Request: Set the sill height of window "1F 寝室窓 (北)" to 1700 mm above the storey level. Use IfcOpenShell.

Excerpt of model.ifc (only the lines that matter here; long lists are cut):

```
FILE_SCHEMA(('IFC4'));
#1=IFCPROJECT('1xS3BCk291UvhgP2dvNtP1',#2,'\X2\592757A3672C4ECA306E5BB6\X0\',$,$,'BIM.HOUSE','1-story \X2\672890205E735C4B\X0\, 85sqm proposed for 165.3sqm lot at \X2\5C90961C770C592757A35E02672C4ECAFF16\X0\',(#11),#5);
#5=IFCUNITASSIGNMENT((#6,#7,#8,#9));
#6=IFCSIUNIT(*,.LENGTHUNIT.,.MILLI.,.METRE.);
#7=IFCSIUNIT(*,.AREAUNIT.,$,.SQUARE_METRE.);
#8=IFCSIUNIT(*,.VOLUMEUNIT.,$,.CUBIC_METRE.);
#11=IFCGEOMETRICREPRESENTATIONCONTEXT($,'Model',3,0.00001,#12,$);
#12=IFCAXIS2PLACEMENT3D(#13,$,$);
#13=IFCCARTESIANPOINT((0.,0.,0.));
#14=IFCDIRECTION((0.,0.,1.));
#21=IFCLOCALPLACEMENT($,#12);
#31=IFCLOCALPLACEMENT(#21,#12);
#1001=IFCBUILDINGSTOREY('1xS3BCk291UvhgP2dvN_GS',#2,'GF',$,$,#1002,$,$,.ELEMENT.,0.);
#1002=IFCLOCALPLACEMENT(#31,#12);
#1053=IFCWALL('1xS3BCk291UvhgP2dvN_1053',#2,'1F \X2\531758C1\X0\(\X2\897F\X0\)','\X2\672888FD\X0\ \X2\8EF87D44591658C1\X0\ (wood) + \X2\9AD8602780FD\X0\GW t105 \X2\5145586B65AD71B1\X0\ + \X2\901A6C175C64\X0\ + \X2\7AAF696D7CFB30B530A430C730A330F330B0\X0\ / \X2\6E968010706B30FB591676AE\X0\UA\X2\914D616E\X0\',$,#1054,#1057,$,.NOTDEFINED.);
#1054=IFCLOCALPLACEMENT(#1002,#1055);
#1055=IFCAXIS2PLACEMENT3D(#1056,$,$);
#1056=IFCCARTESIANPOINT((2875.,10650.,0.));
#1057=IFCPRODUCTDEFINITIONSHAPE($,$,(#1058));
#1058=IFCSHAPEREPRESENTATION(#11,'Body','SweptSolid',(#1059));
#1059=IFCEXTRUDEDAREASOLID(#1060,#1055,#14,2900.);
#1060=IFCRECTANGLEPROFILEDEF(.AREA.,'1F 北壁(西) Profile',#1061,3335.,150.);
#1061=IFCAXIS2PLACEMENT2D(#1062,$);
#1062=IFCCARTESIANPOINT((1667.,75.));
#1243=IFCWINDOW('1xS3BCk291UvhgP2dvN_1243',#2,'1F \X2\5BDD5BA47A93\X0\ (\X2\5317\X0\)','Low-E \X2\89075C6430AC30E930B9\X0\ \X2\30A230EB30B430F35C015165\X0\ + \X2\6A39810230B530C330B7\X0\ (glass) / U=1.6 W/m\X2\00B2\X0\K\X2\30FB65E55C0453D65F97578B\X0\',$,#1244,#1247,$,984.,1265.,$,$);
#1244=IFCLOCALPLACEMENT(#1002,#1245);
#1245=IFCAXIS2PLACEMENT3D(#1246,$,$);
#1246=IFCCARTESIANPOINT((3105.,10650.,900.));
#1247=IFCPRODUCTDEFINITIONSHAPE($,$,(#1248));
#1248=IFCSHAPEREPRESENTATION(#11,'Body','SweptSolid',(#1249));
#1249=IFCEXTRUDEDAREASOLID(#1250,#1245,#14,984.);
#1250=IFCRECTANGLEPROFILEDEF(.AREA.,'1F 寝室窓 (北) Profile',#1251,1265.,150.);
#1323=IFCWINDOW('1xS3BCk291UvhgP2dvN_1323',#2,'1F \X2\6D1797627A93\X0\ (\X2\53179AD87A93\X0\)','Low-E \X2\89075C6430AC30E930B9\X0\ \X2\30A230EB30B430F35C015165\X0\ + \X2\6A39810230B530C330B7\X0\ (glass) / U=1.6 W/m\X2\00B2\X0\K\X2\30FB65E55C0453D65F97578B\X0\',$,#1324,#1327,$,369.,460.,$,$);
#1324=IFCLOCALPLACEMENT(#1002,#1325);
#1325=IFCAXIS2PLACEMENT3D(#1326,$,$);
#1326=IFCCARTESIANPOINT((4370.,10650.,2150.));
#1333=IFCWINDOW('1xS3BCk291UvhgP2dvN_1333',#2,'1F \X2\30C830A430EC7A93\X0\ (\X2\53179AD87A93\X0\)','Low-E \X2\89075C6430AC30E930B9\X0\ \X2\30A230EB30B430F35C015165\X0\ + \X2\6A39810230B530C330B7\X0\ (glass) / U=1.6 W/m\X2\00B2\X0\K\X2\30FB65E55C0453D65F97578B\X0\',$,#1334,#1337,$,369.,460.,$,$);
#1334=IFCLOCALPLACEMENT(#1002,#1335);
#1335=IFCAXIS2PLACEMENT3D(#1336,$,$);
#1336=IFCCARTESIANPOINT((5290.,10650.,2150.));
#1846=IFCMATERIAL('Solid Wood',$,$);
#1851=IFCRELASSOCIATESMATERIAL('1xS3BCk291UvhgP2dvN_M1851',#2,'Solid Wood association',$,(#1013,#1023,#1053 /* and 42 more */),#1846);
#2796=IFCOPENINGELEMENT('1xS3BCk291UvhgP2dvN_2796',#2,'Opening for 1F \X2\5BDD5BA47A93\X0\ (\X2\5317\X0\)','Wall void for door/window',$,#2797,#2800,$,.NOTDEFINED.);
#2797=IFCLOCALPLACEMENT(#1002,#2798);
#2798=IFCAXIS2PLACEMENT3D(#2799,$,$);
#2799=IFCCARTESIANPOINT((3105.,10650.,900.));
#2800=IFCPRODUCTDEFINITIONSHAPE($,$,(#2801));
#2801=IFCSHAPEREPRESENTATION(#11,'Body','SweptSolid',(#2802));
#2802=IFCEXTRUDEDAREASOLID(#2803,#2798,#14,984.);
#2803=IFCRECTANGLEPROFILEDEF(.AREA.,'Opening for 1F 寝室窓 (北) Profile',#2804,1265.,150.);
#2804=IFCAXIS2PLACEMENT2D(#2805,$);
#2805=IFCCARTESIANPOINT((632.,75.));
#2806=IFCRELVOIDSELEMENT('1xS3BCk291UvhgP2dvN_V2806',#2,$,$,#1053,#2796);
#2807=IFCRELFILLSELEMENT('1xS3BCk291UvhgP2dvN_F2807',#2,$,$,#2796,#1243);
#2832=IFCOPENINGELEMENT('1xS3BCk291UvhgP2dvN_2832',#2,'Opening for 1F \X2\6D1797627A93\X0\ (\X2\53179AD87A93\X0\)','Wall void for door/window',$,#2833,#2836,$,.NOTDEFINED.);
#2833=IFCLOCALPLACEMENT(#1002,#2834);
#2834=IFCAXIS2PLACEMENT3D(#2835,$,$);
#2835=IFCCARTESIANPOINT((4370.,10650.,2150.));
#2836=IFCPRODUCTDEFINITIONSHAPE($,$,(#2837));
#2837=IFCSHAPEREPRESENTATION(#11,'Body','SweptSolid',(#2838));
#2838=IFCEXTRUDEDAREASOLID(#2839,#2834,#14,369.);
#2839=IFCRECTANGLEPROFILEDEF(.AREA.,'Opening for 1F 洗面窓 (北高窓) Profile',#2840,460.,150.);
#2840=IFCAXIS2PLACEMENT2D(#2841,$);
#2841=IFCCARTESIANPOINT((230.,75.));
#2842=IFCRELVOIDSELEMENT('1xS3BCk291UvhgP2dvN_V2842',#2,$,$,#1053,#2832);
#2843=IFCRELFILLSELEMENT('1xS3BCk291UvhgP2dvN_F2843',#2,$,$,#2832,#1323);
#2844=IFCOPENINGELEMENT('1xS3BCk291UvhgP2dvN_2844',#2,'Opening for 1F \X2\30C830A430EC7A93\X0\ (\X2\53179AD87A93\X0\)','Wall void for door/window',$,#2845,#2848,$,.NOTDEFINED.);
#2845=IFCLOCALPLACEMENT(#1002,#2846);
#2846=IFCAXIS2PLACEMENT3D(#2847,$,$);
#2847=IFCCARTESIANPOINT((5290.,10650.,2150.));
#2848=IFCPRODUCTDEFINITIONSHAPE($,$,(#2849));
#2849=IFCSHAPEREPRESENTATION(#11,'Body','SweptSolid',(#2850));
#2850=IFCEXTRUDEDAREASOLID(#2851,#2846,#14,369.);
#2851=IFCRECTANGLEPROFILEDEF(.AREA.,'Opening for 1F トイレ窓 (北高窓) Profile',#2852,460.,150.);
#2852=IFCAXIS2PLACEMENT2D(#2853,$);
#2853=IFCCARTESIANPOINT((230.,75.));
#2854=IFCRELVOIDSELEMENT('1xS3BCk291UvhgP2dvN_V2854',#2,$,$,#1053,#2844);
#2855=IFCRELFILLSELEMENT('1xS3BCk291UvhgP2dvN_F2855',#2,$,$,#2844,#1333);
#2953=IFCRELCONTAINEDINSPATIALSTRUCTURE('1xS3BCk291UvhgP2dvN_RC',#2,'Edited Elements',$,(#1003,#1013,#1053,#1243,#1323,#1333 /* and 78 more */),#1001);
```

```python
import numpy as np
import ifcopenshell
import ifcopenshell.api.geometry
import ifcopenshell.geom
import ifcopenshell.util.element
import ifcopenshell.util.placement
import ifcopenshell.util.shape
import ifcopenshell.util.unit

model = ifcopenshell.open("model.ifc")
unit_scale = ifcopenshell.util.unit.calculate_unit_scale(model)

window = model.by_guid("1xS3BCk291UvhgP2dvN_1243")
opening = window.FillsVoids[0].RelatingOpeningElement
storey = ifcopenshell.util.element.get_container(window, ifc_class="IfcBuildingStorey")
level = ifcopenshell.util.placement.get_local_placement(storey.ObjectPlacement)[2, 3]

# The opening's origin need not be at the sill, so measure its lowest point.
shape = ifcopenshell.geom.create_shape(ifcopenshell.geom.settings(), opening)
bottom = ifcopenshell.util.shape.get_shape_bottom_elevation(shape, shape.geometry) / unit_scale
dz = level + 1.7 / unit_scale - bottom

shift = np.array([0.0, 0.0, dz])
# The window is not placed relative to its opening, so move both.
for product in (opening, window):
    matrix = ifcopenshell.util.placement.get_local_placement(product.ObjectPlacement)
    matrix[:3, 3] += shift
    ifcopenshell.api.geometry.edit_object_placement(model, product=product, matrix=matrix, is_si=False)

print(f"moved by {dz * unit_scale:+.3f} m")

model.write("model_updated.ifc")
```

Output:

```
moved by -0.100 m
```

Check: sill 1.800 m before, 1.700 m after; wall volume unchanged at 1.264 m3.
